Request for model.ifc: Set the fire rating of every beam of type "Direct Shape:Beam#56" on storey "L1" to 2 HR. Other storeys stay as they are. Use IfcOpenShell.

First a look at what the model holds.

```python
import ifcopenshell
import ifcopenshell.util.element

model = ifcopenshell.open("model.ifc")
print(model.schema)
storey = next(s for s in model.by_type("IfcBuildingStorey") if s.Name == "L1")
beams = [e for e in ifcopenshell.util.element.get_decomposition(storey) if e.is_a("IfcBeam")]
seen = {}
for e in beams:
    element_type = ifcopenshell.util.element.get_type(e)
    key = (element_type.Name if element_type != e and element_type else None, ifcopenshell.util.element.get_pset(e, "Pset_BeamCommon", "FireRating"))
    seen[key] = seen.get(key, 0) + 1
for (name, value), count in sorted(seen.items(), key=str):
    print(count, "x", name, "|", value)
```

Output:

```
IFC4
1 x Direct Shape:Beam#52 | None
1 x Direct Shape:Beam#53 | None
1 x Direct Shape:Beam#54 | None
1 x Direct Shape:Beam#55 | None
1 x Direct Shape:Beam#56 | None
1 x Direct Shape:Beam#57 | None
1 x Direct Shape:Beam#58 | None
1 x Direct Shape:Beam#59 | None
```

```python
import ifcopenshell
import ifcopenshell.api.pset
import ifcopenshell.util.element

model = ifcopenshell.open("model.ifc")

storey = next(s for s in model.by_type("IfcBuildingStorey") if s.Name == "L1")
beams = [e for e in ifcopenshell.util.element.get_decomposition(storey) if e.is_a("IfcBeam")]

count = 0
for e in beams:
    element_type = ifcopenshell.util.element.get_type(e)
    if element_type in (None, e) or element_type.Name != "Direct Shape:Beam#56":
        continue
    # add_pset returns the element's existing set when there is one.
    pset = ifcopenshell.api.pset.add_pset(model, product=e, name="Pset_BeamCommon")
    ifcopenshell.api.pset.edit_pset(model, pset=pset, properties={"FireRating": "2 HR"})
    count += 1

print(count, "beams updated")

model.write("model-out.ifc")
```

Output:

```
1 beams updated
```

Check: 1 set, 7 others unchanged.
